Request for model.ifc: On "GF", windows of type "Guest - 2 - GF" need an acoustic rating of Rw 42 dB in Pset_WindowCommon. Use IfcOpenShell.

First a look at what the model holds.

```python
import ifcopenshell
import ifcopenshell.util.element

model = ifcopenshell.open("model.ifc")
print(model.schema)
storey = next(s for s in model.by_type("IfcBuildingStorey") if s.Name == "GF")
windows = [e for e in ifcopenshell.util.element.get_decomposition(storey) if e.is_a("IfcWindow")]
seen = {}
for e in windows:
    element_type = ifcopenshell.util.element.get_type(e)
    key = (element_type.Name if element_type != e and element_type else None, ifcopenshell.util.element.get_pset(e, "Pset_WindowCommon", "AcousticRating"))
    seen[key] = seen.get(key, 0) + 1
for (name, value), count in sorted(seen.items(), key=str):
    print(count, "x", name, "|", value)
```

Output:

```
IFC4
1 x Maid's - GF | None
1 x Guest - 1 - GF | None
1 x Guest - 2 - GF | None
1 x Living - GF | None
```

```python
import ifcopenshell
import ifcopenshell.api.pset
import ifcopenshell.util.element

model = ifcopenshell.open("model.ifc")

storey = next(s for s in model.by_type("IfcBuildingStorey") if s.Name == "GF")
windows = [e for e in ifcopenshell.util.element.get_decomposition(storey) if e.is_a("IfcWindow")]

count = 0
for e in windows:
    element_type = ifcopenshell.util.element.get_type(e)
    if element_type in (None, e) or element_type.Name != "Guest - 2 - GF":
        continue
    # add_pset returns the element's existing set when there is one.
    pset = ifcopenshell.api.pset.add_pset(model, product=e, name="Pset_WindowCommon")
    ifcopenshell.api.pset.edit_pset(model, pset=pset, properties={"AcousticRating": "Rw 42 dB"})
    count += 1

print(count, "windows updated")

model.write("model_edited.ifc")
```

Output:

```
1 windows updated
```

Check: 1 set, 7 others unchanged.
